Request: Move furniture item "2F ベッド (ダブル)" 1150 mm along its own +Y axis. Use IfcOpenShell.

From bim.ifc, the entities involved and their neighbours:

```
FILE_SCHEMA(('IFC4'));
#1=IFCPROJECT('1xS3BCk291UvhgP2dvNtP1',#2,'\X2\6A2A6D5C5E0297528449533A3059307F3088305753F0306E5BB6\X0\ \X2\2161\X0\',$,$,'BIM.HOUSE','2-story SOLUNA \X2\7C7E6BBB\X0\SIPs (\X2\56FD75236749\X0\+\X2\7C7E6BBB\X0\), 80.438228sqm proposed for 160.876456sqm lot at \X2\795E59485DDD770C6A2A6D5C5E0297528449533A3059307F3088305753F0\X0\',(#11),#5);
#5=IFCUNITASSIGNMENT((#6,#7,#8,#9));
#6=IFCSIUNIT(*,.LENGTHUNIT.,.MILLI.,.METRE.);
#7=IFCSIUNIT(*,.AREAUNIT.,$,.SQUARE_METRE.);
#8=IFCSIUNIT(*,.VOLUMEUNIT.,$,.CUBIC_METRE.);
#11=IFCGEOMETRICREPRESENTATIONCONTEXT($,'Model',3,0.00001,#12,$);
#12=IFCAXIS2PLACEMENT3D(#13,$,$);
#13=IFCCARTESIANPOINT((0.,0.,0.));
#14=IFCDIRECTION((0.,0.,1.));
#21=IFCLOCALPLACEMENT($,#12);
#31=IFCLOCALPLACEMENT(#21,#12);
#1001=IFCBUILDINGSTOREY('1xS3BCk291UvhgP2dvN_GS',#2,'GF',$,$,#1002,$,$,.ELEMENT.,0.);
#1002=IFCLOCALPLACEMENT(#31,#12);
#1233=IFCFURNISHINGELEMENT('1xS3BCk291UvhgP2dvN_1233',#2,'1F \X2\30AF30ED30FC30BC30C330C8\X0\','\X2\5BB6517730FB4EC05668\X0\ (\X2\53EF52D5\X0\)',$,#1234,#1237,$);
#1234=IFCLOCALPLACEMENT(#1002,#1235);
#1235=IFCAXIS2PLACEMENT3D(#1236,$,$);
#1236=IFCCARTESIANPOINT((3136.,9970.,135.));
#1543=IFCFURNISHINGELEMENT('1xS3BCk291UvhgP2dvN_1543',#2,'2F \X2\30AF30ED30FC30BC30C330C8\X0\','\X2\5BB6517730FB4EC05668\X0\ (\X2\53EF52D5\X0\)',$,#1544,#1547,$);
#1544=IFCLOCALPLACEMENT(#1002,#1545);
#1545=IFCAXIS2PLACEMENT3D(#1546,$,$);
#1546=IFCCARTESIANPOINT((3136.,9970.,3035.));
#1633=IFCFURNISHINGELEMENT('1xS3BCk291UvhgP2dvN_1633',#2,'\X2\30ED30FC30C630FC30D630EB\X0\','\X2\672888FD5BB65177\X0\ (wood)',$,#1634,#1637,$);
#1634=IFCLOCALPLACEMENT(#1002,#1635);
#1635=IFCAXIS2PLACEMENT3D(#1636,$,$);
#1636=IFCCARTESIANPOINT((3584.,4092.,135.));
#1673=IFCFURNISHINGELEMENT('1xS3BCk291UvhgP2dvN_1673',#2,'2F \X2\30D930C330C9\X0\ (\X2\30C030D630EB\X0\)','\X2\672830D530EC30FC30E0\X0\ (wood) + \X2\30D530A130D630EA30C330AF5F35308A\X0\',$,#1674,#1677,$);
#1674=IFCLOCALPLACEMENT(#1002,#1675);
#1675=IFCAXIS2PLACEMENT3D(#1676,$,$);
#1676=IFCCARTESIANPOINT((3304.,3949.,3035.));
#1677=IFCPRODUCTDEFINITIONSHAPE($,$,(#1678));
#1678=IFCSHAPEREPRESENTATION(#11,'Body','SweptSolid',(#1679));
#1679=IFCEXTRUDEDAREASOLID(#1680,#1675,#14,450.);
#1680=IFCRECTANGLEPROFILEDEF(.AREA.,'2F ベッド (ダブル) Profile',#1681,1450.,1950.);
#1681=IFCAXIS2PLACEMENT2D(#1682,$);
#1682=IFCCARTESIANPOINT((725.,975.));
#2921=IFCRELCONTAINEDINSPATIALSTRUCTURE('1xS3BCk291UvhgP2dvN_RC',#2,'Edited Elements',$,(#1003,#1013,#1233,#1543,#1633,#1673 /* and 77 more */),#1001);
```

```python
import ifcopenshell
import ifcopenshell.api.geometry
import ifcopenshell.util.placement
import ifcopenshell.util.unit

model = ifcopenshell.open("bim.ifc")
unit_scale = ifcopenshell.util.unit.calculate_unit_scale(model)

item = model.by_guid("1xS3BCk291UvhgP2dvN_1673")
matrix = ifcopenshell.util.placement.get_local_placement(item.ObjectPlacement)
matrix[:3, 3] += matrix[:3, 1] * 1.15 / unit_scale
ifcopenshell.api.geometry.edit_object_placement(model, product=item, matrix=matrix, is_si=False)

print(ifcopenshell.util.placement.get_local_placement(item.ObjectPlacement).round(3) + 0.0)

model.write("bim_updated.ifc")
```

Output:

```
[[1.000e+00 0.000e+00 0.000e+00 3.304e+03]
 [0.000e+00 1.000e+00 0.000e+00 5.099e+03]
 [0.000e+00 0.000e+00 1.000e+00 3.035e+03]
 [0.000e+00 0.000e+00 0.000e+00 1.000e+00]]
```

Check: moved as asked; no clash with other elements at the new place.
